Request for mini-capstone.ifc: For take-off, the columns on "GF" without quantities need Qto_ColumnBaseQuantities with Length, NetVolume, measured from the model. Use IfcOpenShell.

First a look at what the model holds.

```python
import ifcopenshell
import ifcopenshell.util.element
import ifcopenshell.util.unit

model = ifcopenshell.open("mini-capstone.ifc")
print(model.schema)
for unit_type in ("LENGTHUNIT", "AREAUNIT", "VOLUMEUNIT"):
    print(unit_type, ifcopenshell.util.unit.calculate_unit_scale(model, unit_type))
storey = next(s for s in model.by_type("IfcBuildingStorey") if s.Name == "GF")
columns = [e for e in ifcopenshell.util.element.get_decomposition(storey) if e.is_a("IfcColumn")]
for e in sorted(columns, key=lambda e: e.id()):
    print(e.id(), e.is_a(), e.Name, list(ifcopenshell.util.element.get_psets(e, qtos_only=True)), sep=" | ")
```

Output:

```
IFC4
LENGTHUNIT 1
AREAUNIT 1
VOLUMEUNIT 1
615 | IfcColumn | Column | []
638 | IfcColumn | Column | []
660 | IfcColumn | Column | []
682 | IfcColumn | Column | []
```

```python
import ifcopenshell
import ifcopenshell.api.pset
import ifcopenshell.geom
import ifcopenshell.util.element
import ifcopenshell.util.shape
import ifcopenshell.util.unit

model = ifcopenshell.open("mini-capstone.ifc")
unit_scale = ifcopenshell.util.unit.calculate_unit_scale(model)
volume_scale = ifcopenshell.util.unit.calculate_unit_scale(model, "VOLUMEUNIT")
settings = ifcopenshell.geom.settings()

storey = next(s for s in model.by_type("IfcBuildingStorey") if s.Name == "GF")
columns = [e for e in ifcopenshell.util.element.get_decomposition(storey) if e.is_a("IfcColumn")]

for e in sorted(columns, key=lambda e: e.id()):
    if ifcopenshell.util.element.get_psets(e, qtos_only=True, should_inherit=False):
        continue
    # Geometry comes back in metres, in the element's own axes.
    shape = ifcopenshell.geom.create_shape(settings, e)
    values = {
        "Length": ifcopenshell.util.shape.get_z(shape.geometry) / unit_scale,
        "NetVolume": ifcopenshell.util.shape.get_volume(shape.geometry) / volume_scale,
    }
    qto = ifcopenshell.api.pset.add_qto(model, product=e, name="Qto_ColumnBaseQuantities")
    ifcopenshell.api.pset.edit_qto(model, qto=qto, properties=values)
    print(e.id(), {k: round(v, 3) for k, v in values.items()})

model.write("mini-capstone_rev.ifc")
```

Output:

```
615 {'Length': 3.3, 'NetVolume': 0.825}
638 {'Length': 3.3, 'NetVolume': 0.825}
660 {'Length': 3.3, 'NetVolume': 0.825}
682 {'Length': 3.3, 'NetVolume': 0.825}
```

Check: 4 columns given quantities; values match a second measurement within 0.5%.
